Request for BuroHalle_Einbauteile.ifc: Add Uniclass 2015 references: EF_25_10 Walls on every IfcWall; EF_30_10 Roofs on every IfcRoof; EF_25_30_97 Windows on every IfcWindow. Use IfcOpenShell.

First a look at what the model holds.

```python
import ifcopenshell

model = ifcopenshell.open("BuroHalle_Einbauteile.ifc")
print(model.schema)
print("classifications:", [c.Name for c in model.by_type("IfcClassification")])
for ifc_class in ("IfcDoor", "IfcRoof", "IfcStair", "IfcWall", "IfcWindow"):
    print(ifc_class, len(model.by_type(ifc_class)))
```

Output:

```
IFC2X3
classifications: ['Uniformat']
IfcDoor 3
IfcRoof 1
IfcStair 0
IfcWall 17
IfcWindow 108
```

```python
import ifcopenshell
import ifcopenshell.api.classification

model = ifcopenshell.open("BuroHalle_Einbauteile.ifc")

# IFC2X3 requires Source and Edition and has no link from the project to the system.
system = model.create_entity("IfcClassification", Source="NBS", Edition="2015", Name="Uniclass 2015")

codes = {
    "IfcWall": ("EF_25_10", "Walls"),
    "IfcRoof": ("EF_30_10", "Roofs"),
    "IfcWindow": ("EF_25_30_97", "Windows"),
}
for ifc_class, (code, name) in codes.items():
    products = model.by_type(ifc_class)
    ifcopenshell.api.classification.add_reference(
        model, products=products, classification=system, identification=code, name=name
    )
    print(code, len(products))

model.write("BuroHalle_Einbauteile_v2.ifc")
```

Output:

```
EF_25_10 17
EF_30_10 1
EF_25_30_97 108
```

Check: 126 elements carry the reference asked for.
